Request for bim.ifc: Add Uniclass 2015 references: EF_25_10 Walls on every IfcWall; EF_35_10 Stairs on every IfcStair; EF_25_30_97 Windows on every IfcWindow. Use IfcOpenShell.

First a look at what the model holds.

```python
import ifcopenshell

model = ifcopenshell.open("bim.ifc")
print(model.schema)
print("classifications:", [c.Name for c in model.by_type("IfcClassification")])
for ifc_class in ("IfcDoor", "IfcRoof", "IfcStair", "IfcWall", "IfcWindow"):
    print(ifc_class, len(model.by_type(ifc_class)))
```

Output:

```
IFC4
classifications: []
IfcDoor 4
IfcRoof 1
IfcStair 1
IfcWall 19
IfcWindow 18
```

```python
import ifcopenshell
import ifcopenshell.api.classification

model = ifcopenshell.open("bim.ifc")

system = ifcopenshell.api.classification.add_classification(model, classification="Uniclass 2015")

codes = {
    "IfcWall": ("EF_25_10", "Walls"),
    "IfcStair": ("EF_35_10", "Stairs"),
    "IfcWindow": ("EF_25_30_97", "Windows"),
}
for ifc_class, (code, name) in codes.items():
    products = model.by_type(ifc_class)
    ifcopenshell.api.classification.add_reference(
        model, products=products, classification=system, identification=code, name=name
    )
    print(code, len(products))

model.write("bim_updated.ifc")
```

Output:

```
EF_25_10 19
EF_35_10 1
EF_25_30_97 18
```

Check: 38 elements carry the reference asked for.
